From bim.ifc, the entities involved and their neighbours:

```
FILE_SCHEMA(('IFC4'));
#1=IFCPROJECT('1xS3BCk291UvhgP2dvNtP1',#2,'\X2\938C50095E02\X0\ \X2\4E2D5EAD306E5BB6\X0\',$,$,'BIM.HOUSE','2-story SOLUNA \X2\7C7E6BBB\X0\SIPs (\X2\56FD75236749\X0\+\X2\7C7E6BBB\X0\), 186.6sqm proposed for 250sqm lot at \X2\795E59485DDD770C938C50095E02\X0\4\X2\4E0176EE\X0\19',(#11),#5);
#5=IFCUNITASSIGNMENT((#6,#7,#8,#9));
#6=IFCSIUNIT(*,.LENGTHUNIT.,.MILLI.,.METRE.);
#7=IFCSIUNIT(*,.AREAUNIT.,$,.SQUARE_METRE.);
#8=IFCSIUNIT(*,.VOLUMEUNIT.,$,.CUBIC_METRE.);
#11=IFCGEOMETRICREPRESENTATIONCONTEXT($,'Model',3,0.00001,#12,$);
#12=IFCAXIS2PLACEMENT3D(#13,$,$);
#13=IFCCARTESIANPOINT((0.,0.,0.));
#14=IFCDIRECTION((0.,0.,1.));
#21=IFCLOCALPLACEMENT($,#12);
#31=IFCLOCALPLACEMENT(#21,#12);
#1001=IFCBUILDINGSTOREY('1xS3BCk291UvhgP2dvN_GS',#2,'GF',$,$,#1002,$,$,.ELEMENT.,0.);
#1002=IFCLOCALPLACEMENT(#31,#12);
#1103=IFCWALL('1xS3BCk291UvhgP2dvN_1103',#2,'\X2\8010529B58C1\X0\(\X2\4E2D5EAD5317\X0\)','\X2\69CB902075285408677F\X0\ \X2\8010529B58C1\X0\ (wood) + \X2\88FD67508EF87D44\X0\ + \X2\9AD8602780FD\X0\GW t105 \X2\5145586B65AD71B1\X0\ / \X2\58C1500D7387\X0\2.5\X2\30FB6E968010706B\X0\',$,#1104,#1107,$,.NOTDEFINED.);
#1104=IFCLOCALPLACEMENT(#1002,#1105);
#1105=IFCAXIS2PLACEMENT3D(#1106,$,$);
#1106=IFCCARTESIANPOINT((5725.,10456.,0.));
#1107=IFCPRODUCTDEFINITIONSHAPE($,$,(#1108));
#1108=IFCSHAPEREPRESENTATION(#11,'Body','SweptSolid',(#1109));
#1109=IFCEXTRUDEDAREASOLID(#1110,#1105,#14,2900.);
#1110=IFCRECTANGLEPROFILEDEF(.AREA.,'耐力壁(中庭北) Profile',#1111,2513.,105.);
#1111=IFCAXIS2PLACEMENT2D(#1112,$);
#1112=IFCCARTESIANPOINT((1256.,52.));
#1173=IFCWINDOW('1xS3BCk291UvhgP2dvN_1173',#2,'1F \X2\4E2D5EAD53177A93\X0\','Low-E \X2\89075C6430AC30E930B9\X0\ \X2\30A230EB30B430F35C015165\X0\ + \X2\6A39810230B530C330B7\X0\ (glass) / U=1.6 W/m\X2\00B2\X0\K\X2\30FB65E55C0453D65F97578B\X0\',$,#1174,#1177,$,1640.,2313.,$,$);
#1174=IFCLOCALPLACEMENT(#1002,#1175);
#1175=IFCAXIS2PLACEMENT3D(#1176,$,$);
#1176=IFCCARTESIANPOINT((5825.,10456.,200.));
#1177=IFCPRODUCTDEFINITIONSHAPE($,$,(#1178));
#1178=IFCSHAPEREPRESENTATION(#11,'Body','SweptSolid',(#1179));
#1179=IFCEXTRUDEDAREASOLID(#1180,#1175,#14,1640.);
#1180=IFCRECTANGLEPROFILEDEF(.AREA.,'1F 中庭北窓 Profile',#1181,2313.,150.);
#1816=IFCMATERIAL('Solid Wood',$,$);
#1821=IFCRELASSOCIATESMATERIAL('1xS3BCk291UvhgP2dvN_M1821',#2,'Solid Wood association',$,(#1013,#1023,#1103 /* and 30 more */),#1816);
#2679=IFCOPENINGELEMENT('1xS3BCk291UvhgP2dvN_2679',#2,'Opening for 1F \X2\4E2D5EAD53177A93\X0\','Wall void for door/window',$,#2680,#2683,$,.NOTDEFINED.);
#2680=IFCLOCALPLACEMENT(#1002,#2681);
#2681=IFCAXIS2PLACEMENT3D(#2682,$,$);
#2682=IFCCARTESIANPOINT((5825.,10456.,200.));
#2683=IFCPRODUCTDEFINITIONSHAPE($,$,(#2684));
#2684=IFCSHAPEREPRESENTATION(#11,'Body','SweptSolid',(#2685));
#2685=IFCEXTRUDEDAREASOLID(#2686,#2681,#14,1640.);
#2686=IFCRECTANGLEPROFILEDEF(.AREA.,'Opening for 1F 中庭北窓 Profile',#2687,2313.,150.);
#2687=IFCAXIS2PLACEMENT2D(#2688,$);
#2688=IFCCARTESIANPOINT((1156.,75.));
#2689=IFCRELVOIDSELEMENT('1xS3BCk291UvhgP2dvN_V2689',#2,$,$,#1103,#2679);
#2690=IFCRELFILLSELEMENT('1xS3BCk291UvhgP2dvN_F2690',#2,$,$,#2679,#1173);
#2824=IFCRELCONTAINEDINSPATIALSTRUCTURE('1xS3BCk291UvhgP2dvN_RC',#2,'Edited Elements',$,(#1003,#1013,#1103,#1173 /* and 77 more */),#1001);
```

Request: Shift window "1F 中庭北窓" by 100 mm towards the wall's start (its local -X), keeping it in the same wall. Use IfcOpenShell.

```python
import ifcopenshell
import ifcopenshell.api.geometry
import ifcopenshell.util.placement
import ifcopenshell.util.unit

model = ifcopenshell.open("bim.ifc")
unit_scale = ifcopenshell.util.unit.calculate_unit_scale(model)

window = model.by_guid("1xS3BCk291UvhgP2dvN_1173")
opening = window.FillsVoids[0].RelatingOpeningElement
wall = opening.VoidsElements[0].RelatingBuildingElement

wall_matrix = ifcopenshell.util.placement.get_local_placement(wall.ObjectPlacement)
shift = wall_matrix[:3, 0] * -0.1 / unit_scale
before = ifcopenshell.util.placement.get_local_placement(window.ObjectPlacement)[:3, 3].copy()

# The window is not placed relative to its opening, so move both.
for product in (opening, window):
    matrix = ifcopenshell.util.placement.get_local_placement(product.ObjectPlacement)
    matrix[:3, 3] += shift
    ifcopenshell.api.geometry.edit_object_placement(model, product=product, matrix=matrix, is_si=False)

after = ifcopenshell.util.placement.get_local_placement(window.ObjectPlacement)[:3, 3]
print("window moved by", (after - before).round(3) + 0.0)

model.write("bim-out.ifc")
```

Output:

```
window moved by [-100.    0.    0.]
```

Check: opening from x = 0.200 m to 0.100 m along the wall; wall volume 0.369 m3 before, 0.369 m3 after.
